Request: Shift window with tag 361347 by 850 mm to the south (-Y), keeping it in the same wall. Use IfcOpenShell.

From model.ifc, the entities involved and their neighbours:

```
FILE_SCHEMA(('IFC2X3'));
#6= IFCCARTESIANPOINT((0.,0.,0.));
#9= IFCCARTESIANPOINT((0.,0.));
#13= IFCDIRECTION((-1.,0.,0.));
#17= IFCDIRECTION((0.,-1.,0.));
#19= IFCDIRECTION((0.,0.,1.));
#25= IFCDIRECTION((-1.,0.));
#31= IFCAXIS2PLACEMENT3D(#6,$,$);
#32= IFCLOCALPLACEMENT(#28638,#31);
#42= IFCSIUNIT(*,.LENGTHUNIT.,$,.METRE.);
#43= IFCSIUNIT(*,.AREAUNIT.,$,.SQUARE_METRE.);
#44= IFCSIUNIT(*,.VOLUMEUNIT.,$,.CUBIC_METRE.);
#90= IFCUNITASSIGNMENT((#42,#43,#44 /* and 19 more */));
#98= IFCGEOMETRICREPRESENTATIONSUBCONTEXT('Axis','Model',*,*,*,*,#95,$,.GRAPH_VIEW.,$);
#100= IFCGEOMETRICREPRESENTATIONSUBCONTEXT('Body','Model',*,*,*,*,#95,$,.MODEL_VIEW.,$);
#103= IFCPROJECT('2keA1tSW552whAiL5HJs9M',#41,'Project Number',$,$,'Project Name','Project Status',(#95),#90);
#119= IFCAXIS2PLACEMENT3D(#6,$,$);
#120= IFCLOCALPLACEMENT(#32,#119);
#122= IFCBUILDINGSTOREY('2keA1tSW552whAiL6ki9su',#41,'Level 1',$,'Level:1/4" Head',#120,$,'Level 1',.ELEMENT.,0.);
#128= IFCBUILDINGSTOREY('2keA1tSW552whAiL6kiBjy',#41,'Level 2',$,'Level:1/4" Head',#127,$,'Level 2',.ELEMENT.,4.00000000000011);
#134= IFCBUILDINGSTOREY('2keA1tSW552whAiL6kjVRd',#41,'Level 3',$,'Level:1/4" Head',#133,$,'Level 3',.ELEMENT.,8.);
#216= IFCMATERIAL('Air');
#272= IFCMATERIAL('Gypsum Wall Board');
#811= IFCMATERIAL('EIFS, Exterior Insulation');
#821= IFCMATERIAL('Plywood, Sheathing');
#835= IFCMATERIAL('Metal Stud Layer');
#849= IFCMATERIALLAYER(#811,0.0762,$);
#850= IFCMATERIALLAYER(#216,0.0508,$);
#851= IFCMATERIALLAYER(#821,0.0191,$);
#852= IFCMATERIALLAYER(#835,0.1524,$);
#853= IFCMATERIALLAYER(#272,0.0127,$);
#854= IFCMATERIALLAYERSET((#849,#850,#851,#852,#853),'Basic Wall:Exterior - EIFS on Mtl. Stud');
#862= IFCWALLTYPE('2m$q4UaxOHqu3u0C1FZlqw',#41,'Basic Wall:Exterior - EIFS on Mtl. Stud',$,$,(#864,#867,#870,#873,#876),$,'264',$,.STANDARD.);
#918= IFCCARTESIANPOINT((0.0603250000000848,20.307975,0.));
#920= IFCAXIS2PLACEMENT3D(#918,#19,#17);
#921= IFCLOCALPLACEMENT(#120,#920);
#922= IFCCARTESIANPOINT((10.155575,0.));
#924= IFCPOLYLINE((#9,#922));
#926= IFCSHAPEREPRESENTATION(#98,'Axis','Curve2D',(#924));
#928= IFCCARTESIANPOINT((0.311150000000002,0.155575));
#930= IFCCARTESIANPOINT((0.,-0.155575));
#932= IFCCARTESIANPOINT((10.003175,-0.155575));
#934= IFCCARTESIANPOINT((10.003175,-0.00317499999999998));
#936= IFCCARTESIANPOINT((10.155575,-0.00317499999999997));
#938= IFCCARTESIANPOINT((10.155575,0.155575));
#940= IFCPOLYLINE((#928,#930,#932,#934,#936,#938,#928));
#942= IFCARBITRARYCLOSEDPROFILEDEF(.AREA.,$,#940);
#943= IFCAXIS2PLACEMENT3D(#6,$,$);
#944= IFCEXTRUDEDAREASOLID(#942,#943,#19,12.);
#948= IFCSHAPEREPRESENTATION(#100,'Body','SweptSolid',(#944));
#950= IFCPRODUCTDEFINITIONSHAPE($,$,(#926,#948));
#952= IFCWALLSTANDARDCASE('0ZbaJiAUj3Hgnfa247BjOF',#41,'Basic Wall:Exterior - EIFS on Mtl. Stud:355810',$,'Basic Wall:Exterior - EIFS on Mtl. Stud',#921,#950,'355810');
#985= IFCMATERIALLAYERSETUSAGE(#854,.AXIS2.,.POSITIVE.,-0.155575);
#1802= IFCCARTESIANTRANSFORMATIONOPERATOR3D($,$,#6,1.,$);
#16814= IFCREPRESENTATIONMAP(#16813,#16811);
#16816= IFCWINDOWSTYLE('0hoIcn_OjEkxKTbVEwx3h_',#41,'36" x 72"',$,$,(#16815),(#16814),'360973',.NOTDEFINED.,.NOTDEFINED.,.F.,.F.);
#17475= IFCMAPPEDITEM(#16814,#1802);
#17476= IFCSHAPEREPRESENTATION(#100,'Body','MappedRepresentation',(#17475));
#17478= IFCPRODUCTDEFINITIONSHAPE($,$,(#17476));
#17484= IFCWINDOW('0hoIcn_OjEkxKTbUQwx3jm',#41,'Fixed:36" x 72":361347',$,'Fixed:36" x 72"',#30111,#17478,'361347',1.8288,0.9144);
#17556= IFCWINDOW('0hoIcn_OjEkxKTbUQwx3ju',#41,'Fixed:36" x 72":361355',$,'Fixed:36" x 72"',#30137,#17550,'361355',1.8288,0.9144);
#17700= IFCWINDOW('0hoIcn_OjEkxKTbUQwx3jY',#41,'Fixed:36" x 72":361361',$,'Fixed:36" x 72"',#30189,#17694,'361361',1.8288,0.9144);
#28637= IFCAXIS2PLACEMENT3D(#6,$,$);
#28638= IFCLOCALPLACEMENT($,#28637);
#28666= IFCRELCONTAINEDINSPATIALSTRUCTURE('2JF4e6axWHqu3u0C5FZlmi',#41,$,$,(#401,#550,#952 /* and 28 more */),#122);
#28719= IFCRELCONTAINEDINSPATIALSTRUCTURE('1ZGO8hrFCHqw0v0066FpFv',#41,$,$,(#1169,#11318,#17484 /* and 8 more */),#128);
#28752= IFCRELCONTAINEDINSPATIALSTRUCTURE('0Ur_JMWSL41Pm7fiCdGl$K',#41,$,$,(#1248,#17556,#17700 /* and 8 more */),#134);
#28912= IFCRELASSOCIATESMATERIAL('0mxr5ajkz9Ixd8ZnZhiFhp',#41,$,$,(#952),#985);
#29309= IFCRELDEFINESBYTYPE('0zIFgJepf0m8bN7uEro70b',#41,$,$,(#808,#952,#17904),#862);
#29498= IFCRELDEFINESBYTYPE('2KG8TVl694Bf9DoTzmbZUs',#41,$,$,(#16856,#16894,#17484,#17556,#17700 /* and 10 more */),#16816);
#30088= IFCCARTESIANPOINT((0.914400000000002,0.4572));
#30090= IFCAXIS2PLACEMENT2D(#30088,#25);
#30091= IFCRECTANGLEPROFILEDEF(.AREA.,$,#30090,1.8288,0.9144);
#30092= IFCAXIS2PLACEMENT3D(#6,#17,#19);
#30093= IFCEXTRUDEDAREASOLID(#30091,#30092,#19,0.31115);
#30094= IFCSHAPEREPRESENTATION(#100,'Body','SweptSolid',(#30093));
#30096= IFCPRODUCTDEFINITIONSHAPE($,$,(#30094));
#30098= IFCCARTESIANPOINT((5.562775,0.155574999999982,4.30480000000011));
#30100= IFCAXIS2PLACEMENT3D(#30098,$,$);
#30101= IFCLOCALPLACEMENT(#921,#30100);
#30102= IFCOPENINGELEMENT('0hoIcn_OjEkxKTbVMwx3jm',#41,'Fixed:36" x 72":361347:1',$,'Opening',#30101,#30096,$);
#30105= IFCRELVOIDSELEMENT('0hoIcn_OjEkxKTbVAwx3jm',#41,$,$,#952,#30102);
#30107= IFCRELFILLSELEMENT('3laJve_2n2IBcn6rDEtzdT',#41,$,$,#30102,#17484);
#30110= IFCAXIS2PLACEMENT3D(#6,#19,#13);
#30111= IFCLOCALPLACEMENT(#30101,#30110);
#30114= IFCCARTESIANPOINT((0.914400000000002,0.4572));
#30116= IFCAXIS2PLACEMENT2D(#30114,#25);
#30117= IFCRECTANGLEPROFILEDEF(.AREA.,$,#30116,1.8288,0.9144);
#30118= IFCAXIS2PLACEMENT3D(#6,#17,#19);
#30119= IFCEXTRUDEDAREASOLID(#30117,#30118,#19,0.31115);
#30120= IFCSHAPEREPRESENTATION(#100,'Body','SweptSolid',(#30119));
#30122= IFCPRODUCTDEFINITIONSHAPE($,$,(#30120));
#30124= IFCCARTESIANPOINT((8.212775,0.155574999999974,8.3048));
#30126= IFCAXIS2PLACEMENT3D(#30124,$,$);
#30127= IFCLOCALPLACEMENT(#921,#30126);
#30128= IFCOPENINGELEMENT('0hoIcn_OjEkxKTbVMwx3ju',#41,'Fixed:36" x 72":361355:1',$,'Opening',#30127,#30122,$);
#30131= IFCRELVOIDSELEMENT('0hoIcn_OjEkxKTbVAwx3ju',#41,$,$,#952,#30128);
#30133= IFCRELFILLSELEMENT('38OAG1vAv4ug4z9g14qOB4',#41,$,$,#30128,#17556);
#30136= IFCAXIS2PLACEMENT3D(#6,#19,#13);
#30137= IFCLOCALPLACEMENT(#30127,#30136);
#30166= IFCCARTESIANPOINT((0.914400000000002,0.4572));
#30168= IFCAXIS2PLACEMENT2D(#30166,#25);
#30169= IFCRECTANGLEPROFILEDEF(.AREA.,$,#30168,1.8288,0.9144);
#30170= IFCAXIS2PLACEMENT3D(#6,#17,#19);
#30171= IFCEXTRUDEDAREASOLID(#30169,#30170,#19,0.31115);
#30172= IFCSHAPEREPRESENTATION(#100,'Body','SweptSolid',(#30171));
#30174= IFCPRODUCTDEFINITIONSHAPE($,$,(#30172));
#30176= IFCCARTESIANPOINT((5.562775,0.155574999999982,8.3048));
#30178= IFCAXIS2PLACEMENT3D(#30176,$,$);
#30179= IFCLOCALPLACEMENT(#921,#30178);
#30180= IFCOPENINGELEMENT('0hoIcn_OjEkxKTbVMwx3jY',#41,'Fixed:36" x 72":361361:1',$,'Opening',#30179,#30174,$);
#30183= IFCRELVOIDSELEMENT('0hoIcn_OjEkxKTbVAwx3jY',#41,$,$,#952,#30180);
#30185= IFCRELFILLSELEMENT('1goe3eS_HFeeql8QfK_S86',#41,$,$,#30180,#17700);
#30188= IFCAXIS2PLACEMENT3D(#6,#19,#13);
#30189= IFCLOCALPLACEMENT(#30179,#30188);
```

```python
import ifcopenshell
import ifcopenshell.api.geometry
import ifcopenshell.util.placement
import ifcopenshell.util.unit

model = ifcopenshell.open("model.ifc")
unit_scale = ifcopenshell.util.unit.calculate_unit_scale(model)

window = model.by_guid("0hoIcn_OjEkxKTbUQwx3jm")
opening = window.FillsVoids[0].RelatingOpeningElement
wall = opening.VoidsElements[0].RelatingBuildingElement

wall_matrix = ifcopenshell.util.placement.get_local_placement(wall.ObjectPlacement)
shift = wall_matrix[:3, 0] * 0.85 / unit_scale
before = ifcopenshell.util.placement.get_local_placement(window.ObjectPlacement)[:3, 3].copy()

# The window is placed relative to its opening, so it follows when the opening moves.
matrix = ifcopenshell.util.placement.get_local_placement(opening.ObjectPlacement)
matrix[:3, 3] += shift
ifcopenshell.api.geometry.edit_object_placement(
    model, product=opening, matrix=matrix, is_si=False, should_transform_children=True
)

after = ifcopenshell.util.placement.get_local_placement(window.ObjectPlacement)[:3, 3]
print("window moved by", (after - before).round(3) + 0.0)

model.write("model-out.ifc")
```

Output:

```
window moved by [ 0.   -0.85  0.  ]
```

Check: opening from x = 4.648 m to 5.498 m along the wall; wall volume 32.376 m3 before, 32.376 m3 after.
